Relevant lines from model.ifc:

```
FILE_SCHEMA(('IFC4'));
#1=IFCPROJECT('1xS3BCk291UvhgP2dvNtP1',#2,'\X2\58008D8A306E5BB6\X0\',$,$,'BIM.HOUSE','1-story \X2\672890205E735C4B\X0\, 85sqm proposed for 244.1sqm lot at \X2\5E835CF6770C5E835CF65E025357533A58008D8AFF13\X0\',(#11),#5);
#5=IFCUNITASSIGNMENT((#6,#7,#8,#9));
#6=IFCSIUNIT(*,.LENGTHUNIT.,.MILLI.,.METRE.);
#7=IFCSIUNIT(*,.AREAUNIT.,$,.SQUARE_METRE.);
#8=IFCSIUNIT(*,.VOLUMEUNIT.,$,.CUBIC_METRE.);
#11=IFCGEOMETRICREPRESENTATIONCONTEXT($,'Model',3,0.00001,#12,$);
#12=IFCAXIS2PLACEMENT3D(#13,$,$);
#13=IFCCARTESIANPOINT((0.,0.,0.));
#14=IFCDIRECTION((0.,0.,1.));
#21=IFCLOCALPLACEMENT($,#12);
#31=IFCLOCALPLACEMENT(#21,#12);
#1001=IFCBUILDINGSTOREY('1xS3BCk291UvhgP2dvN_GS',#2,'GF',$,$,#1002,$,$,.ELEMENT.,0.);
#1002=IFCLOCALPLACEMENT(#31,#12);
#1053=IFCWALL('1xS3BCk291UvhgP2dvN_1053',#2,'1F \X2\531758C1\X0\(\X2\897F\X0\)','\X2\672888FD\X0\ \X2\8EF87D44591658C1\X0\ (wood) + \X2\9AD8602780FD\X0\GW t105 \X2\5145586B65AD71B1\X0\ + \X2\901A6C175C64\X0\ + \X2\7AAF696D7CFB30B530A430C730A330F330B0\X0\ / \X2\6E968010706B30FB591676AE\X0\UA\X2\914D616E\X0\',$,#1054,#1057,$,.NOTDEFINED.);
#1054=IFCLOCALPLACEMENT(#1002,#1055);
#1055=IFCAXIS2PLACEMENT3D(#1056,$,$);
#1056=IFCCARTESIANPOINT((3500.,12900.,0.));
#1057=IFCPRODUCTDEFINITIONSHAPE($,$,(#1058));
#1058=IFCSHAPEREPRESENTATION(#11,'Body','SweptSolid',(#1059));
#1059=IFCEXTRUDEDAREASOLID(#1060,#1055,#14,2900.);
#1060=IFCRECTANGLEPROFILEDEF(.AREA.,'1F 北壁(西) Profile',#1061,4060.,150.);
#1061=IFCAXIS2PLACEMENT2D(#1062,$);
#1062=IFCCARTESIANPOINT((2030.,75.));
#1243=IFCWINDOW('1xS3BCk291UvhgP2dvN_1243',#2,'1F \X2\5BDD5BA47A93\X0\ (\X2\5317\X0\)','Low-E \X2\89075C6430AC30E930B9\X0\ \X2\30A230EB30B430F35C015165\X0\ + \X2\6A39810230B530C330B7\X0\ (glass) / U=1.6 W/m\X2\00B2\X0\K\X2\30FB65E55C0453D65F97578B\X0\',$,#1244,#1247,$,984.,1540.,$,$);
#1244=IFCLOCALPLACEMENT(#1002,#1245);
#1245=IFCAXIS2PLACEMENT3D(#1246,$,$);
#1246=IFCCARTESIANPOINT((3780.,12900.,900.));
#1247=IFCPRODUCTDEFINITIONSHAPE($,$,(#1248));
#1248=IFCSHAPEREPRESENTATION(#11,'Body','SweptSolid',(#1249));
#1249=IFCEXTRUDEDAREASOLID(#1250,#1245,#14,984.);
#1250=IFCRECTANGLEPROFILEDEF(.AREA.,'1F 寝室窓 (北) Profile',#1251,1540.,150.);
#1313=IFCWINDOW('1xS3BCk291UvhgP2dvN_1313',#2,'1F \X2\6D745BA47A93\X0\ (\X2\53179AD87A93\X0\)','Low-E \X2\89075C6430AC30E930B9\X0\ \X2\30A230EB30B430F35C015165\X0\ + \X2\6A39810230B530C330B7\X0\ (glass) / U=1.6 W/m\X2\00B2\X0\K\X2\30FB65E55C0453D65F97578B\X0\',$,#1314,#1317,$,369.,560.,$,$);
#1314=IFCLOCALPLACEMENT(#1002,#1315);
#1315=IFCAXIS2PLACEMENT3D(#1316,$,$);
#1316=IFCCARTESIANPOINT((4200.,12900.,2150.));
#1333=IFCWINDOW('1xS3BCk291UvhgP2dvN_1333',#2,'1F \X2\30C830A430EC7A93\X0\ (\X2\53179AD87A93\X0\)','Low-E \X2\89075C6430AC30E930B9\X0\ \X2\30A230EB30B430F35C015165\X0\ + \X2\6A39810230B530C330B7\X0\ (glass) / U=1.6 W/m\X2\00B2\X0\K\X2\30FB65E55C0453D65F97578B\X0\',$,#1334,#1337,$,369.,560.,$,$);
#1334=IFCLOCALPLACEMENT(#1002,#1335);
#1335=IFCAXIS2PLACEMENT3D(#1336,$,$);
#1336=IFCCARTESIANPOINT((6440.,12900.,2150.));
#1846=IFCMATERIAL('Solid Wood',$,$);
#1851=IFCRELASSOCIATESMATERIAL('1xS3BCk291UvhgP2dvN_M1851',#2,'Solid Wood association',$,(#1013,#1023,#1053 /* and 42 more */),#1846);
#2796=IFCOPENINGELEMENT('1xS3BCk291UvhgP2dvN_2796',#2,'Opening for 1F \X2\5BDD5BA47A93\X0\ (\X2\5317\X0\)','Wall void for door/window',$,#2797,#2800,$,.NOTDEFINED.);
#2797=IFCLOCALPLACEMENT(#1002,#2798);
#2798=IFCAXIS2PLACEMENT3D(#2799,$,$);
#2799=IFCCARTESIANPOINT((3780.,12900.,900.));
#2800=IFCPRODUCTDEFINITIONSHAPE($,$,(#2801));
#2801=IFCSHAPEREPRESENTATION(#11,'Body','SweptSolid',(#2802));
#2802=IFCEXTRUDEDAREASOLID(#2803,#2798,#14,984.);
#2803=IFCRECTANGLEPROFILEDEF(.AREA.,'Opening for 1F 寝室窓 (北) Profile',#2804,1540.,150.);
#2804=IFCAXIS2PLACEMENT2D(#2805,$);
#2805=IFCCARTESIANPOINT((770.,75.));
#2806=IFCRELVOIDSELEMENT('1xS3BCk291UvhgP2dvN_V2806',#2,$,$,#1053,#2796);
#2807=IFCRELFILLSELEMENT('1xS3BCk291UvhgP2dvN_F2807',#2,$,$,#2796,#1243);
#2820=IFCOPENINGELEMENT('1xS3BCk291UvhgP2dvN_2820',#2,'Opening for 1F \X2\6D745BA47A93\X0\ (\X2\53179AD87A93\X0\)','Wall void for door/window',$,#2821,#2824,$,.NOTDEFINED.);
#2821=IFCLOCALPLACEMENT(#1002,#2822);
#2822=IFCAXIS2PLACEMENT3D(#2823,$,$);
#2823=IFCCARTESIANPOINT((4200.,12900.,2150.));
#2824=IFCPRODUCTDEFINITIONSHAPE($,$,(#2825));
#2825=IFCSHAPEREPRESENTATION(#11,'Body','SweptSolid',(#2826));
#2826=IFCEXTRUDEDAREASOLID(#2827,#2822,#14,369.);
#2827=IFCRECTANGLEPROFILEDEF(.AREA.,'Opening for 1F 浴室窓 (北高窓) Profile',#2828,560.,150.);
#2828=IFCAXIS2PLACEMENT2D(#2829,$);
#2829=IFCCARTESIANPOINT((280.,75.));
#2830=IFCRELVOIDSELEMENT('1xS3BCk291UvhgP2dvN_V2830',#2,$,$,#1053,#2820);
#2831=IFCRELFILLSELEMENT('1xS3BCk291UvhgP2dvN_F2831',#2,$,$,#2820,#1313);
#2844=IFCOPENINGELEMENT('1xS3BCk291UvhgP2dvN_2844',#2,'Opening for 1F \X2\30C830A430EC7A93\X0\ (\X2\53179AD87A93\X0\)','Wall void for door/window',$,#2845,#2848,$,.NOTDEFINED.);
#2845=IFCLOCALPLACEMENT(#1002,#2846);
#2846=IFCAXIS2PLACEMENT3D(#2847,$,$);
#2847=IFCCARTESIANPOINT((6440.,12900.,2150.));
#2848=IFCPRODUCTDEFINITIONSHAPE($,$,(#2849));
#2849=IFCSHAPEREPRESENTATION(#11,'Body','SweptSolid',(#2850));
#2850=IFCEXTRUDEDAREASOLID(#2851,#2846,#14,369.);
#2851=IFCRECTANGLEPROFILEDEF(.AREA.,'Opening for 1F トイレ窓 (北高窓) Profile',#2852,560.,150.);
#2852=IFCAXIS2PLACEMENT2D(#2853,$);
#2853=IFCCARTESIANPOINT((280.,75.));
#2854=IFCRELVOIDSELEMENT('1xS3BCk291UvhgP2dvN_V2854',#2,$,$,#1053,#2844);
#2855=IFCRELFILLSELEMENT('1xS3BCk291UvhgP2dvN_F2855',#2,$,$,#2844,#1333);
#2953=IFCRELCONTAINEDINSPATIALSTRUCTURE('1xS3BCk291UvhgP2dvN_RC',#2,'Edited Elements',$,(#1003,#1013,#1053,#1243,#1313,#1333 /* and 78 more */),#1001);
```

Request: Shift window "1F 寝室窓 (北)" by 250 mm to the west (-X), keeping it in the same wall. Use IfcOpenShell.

```python
import ifcopenshell
import ifcopenshell.api.geometry
import ifcopenshell.util.placement

model = ifcopenshell.open("model.ifc")

window = model.by_id(1243)
opening = window.FillsVoids[0].RelatingOpeningElement
wall = opening.VoidsElements[0].RelatingBuildingElement

wall_matrix = ifcopenshell.util.placement.get_local_placement(wall.ObjectPlacement)
shift = wall_matrix[:3, 0] * -250.0
before = ifcopenshell.util.placement.get_local_placement(window.ObjectPlacement)[:3, 3].copy()

# The window is not placed relative to its opening, so move both.
for product in (opening, window):
    matrix = ifcopenshell.util.placement.get_local_placement(product.ObjectPlacement)
    matrix[:3, 3] += shift
    ifcopenshell.api.geometry.edit_object_placement(model, product=product, matrix=matrix, is_si=False)

after = ifcopenshell.util.placement.get_local_placement(window.ObjectPlacement)[:3, 3]
print("window moved by", (after - before).round(3) + 0.0)

model.write("model_v2.ifc")
```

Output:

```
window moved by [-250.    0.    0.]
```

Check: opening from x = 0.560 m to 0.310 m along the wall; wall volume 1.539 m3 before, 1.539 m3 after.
